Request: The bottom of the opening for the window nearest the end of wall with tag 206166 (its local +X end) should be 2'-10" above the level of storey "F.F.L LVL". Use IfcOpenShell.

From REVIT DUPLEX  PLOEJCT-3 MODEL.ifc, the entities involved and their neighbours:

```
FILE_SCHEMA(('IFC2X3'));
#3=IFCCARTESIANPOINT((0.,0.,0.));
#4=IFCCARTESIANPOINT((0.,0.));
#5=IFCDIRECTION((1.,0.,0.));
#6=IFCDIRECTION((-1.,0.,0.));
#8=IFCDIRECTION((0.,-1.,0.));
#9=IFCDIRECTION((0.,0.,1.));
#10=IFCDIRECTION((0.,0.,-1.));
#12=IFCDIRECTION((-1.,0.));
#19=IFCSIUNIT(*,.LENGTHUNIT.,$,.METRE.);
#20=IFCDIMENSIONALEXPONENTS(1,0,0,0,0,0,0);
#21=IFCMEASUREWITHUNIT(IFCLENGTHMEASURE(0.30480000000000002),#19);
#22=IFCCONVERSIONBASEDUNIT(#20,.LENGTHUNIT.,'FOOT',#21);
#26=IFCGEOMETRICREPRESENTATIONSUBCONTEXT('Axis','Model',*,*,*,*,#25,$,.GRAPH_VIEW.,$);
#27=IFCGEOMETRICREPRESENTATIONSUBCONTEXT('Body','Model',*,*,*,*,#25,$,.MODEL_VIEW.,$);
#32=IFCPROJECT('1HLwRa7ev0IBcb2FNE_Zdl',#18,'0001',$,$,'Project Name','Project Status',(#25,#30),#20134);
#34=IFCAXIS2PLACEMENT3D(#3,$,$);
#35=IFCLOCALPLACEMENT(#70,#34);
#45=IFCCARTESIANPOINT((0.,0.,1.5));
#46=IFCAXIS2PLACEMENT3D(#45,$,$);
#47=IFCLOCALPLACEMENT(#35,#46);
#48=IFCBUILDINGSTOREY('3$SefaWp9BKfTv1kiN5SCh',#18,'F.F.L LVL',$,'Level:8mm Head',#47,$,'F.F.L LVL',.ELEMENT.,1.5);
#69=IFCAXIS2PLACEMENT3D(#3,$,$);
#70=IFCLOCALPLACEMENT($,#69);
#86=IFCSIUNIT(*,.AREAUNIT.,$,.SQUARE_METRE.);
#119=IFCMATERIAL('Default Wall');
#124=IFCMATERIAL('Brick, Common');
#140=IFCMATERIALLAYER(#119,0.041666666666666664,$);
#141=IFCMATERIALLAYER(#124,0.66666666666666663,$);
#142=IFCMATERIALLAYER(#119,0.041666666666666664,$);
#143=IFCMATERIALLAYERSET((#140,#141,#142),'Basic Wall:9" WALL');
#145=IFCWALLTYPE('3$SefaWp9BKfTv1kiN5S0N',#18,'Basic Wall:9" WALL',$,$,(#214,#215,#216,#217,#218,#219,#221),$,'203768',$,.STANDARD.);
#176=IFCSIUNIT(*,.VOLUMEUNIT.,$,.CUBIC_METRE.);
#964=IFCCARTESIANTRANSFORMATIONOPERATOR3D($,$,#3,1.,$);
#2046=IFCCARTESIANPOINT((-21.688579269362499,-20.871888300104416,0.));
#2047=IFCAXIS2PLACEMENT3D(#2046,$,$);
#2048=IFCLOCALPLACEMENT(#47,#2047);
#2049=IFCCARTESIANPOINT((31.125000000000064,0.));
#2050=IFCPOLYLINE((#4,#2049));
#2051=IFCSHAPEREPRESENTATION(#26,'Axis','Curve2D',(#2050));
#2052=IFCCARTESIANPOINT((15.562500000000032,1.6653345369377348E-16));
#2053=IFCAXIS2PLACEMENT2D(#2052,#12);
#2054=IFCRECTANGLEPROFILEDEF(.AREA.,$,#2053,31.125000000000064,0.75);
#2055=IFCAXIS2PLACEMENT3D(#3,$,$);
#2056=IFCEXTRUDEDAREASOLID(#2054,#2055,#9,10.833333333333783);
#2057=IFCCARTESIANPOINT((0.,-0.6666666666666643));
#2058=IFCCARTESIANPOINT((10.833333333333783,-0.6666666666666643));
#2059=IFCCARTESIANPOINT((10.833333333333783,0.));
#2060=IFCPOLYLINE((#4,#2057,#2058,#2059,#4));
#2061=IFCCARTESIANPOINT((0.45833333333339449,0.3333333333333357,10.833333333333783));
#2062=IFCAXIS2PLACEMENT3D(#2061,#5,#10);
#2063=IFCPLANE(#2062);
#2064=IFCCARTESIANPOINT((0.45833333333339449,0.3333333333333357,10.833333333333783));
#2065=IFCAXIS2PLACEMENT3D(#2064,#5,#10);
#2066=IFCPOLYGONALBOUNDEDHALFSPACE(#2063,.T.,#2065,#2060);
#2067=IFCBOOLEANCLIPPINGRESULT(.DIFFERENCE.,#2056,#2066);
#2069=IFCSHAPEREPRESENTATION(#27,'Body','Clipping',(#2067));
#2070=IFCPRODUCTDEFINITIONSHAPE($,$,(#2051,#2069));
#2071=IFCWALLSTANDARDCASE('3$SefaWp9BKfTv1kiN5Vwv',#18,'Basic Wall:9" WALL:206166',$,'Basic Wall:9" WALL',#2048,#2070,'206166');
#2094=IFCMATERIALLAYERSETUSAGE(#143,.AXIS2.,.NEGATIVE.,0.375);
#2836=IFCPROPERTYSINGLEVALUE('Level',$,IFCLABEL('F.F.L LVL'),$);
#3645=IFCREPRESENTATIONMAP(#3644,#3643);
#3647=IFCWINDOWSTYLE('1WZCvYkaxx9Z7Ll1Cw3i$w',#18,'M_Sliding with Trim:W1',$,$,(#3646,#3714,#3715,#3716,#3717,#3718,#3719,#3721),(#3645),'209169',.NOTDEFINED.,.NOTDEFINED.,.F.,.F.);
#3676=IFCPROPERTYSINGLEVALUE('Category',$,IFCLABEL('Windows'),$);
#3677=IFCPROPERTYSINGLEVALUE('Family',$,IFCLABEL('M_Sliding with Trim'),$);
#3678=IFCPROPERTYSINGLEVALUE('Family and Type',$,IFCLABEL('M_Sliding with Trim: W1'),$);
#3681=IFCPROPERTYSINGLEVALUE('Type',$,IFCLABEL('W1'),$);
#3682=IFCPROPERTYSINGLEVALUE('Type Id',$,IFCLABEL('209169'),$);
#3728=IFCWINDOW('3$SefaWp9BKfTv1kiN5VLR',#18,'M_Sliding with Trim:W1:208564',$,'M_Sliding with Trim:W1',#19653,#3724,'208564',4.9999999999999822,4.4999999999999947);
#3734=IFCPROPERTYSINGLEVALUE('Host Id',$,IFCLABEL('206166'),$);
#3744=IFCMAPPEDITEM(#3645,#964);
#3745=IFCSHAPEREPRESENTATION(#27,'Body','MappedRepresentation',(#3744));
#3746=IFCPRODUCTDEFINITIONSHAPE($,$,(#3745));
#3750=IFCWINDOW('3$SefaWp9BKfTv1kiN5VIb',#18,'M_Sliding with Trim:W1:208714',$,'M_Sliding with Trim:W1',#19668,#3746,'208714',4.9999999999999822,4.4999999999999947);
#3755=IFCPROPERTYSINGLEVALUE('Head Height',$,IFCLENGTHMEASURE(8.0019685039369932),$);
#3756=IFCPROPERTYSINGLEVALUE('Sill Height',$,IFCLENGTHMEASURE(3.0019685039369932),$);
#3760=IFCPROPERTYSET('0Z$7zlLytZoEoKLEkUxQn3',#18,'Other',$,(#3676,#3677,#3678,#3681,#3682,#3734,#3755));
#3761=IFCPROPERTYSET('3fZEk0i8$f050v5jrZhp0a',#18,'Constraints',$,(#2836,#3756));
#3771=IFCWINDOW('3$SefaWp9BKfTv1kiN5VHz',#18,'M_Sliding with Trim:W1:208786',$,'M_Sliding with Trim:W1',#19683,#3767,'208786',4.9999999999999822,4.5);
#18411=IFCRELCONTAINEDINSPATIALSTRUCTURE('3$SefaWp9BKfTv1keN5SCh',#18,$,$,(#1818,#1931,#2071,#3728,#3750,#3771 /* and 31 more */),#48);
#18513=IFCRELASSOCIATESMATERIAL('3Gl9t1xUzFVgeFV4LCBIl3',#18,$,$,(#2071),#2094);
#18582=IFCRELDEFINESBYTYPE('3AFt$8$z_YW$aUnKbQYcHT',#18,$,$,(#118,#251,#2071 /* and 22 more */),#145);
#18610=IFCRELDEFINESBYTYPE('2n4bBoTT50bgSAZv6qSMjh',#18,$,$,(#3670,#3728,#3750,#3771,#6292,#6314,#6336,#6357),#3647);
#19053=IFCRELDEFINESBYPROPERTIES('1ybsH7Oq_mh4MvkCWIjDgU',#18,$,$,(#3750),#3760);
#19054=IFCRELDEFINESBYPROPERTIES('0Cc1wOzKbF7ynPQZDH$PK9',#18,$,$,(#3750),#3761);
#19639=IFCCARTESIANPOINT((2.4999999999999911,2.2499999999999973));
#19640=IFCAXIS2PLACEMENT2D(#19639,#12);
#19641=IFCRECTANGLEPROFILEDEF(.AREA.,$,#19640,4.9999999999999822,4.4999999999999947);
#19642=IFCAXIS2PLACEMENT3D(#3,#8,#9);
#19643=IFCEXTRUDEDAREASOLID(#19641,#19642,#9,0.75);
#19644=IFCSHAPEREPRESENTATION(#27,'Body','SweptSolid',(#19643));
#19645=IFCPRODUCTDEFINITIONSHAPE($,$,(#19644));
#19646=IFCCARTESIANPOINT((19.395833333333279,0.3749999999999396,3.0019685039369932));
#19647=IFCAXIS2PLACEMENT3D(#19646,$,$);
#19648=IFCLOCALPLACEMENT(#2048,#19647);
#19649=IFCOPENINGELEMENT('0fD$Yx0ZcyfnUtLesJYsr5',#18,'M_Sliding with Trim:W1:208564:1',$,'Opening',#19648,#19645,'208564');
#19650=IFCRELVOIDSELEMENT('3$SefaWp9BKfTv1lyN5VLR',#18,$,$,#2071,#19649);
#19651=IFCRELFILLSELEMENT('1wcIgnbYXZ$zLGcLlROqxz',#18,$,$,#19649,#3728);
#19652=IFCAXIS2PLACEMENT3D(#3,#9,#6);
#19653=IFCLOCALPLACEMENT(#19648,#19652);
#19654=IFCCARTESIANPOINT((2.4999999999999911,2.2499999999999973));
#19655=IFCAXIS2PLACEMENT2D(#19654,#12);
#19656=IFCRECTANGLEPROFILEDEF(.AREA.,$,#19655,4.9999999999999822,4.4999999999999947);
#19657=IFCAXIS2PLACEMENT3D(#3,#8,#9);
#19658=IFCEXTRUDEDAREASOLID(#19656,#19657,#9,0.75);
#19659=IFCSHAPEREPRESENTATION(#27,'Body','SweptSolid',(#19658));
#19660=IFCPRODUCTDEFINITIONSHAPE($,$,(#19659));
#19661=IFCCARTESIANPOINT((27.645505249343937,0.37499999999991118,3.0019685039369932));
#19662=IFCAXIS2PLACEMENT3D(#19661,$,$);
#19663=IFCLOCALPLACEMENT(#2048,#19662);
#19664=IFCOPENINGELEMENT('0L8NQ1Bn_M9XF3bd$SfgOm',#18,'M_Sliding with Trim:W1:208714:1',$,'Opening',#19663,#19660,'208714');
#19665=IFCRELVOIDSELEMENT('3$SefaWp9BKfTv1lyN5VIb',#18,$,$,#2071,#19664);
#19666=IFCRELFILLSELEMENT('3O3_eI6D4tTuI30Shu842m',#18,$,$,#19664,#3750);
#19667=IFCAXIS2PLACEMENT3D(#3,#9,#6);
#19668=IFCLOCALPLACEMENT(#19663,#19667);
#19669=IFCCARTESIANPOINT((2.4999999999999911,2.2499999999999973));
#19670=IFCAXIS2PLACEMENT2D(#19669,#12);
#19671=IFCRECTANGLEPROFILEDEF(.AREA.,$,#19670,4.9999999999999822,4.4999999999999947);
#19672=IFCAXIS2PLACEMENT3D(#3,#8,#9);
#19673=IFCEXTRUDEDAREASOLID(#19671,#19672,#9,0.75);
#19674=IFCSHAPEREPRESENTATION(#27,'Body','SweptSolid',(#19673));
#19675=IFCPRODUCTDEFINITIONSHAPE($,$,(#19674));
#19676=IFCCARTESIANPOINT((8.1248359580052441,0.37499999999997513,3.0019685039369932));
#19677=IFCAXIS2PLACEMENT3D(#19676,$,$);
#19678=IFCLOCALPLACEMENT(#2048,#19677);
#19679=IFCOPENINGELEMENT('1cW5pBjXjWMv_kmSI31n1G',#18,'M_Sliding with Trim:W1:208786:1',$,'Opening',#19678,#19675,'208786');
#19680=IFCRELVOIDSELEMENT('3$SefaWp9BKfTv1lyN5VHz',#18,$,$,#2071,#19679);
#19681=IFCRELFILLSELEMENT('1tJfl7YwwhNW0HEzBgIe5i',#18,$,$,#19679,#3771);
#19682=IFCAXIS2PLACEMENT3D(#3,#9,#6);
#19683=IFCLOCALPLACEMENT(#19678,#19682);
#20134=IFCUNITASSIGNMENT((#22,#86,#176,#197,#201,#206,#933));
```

```python
import numpy as np
import ifcopenshell
import ifcopenshell.api.geometry
import ifcopenshell.api.pset
import ifcopenshell.geom
import ifcopenshell.util.element
import ifcopenshell.util.placement
import ifcopenshell.util.shape
import ifcopenshell.util.unit

model = ifcopenshell.open("REVIT DUPLEX  PLOEJCT-3 MODEL.ifc")
unit_scale = ifcopenshell.util.unit.calculate_unit_scale(model)

window = model.by_id(3750)
opening = window.FillsVoids[0].RelatingOpeningElement
storey = ifcopenshell.util.element.get_container(window, ifc_class="IfcBuildingStorey")
level = ifcopenshell.util.placement.get_local_placement(storey.ObjectPlacement)[2, 3]

# The opening's origin need not be at the sill, so measure its lowest point.
shape = ifcopenshell.geom.create_shape(ifcopenshell.geom.settings(), opening)
bottom = ifcopenshell.util.shape.get_shape_bottom_elevation(shape, shape.geometry) / unit_scale
dz = level + 34 * 0.0254 / unit_scale - bottom

shift = np.array([0.0, 0.0, dz])
# The window is placed relative to its opening, so it follows when the opening moves.
matrix = ifcopenshell.util.placement.get_local_placement(opening.ObjectPlacement)
matrix[:3, 3] += shift
ifcopenshell.api.geometry.edit_object_placement(
    model, product=opening, matrix=matrix, is_si=False, should_transform_children=True
)

# Keep the stored heights in step.
pset = model.by_id(ifcopenshell.util.element.get_pset(window, "Other", should_inherit=False)["id"])
ifcopenshell.api.pset.edit_pset(model, pset=pset, properties={
    "Head Height": model.create_entity("IfcLengthMeasure", ifcopenshell.util.element.get_pset(window, "Other", "Head Height") + dz),
})
pset = model.by_id(ifcopenshell.util.element.get_pset(window, "Constraints", should_inherit=False)["id"])
ifcopenshell.api.pset.edit_pset(model, pset=pset, properties={
    "Sill Height": model.create_entity("IfcLengthMeasure", ifcopenshell.util.element.get_pset(window, "Constraints", "Sill Height") + dz),
})

print(f"moved by {dz * unit_scale:+.3f} m")

model.write("REVIT DUPLEX  PLOEJCT-3 MODEL_edited.ifc")
```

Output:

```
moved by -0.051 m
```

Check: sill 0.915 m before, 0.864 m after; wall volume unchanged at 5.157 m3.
